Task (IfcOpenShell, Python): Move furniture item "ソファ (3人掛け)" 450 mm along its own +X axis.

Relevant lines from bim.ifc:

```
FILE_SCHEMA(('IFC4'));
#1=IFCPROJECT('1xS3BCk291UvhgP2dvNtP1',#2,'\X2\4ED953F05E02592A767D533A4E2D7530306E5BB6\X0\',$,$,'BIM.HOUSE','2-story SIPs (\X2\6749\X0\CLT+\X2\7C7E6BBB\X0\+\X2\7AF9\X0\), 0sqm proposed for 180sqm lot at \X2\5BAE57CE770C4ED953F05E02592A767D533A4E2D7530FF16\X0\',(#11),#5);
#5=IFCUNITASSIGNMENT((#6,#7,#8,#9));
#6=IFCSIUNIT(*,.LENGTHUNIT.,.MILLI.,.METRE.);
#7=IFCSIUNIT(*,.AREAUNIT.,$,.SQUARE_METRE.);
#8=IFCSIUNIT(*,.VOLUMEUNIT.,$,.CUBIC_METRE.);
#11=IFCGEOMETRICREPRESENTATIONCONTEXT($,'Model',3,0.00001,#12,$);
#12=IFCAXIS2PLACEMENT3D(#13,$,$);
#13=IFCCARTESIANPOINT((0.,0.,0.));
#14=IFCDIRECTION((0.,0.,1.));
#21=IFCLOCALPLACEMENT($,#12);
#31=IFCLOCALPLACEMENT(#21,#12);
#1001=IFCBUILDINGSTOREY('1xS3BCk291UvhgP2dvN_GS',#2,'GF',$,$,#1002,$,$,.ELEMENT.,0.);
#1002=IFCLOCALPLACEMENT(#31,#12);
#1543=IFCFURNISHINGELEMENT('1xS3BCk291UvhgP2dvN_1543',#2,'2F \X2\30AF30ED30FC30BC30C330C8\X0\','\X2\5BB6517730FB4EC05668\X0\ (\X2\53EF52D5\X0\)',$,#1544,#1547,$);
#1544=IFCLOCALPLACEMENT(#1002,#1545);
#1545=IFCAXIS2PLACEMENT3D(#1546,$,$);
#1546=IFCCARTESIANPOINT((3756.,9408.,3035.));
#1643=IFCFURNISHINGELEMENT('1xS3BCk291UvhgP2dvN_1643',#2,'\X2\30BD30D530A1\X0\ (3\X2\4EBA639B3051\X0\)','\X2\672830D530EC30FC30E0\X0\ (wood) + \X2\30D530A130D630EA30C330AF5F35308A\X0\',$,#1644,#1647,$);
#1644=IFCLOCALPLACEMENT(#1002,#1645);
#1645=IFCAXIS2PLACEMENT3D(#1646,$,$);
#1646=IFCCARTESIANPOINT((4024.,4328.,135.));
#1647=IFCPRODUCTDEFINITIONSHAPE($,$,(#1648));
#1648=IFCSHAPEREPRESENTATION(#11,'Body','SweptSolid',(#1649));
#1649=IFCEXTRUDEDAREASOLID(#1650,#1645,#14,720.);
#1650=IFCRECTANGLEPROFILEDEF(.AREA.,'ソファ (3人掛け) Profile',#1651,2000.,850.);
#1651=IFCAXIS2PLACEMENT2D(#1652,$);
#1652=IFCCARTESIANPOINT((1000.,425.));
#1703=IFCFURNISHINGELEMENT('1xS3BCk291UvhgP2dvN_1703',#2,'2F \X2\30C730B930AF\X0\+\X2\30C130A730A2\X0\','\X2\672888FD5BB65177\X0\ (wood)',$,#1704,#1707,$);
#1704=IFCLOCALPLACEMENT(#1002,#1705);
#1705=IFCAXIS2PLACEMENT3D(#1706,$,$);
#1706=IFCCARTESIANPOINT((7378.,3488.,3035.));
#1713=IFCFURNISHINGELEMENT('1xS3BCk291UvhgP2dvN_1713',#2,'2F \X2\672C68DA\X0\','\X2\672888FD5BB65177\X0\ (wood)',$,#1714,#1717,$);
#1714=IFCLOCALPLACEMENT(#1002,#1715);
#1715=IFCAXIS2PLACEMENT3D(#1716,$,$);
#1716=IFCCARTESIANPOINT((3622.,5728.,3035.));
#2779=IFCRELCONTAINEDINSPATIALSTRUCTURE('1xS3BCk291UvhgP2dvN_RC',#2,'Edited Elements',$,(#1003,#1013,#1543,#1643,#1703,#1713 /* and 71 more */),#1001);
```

```python
import ifcopenshell
import ifcopenshell.api.geometry
import ifcopenshell.util.placement
import ifcopenshell.util.unit

model = ifcopenshell.open("bim.ifc")
unit_scale = ifcopenshell.util.unit.calculate_unit_scale(model)

item = model.by_guid("1xS3BCk291UvhgP2dvN_1643")
matrix = ifcopenshell.util.placement.get_local_placement(item.ObjectPlacement)
matrix[:3, 3] += matrix[:3, 0] * 0.45 / unit_scale
ifcopenshell.api.geometry.edit_object_placement(model, product=item, matrix=matrix, is_si=False)

print(ifcopenshell.util.placement.get_local_placement(item.ObjectPlacement).round(3) + 0.0)

model.write("bim-out.ifc")
```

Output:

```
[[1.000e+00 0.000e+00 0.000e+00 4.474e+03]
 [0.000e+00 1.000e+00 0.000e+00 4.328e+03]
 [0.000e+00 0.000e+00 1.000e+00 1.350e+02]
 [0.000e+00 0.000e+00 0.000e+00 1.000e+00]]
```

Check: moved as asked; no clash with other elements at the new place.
